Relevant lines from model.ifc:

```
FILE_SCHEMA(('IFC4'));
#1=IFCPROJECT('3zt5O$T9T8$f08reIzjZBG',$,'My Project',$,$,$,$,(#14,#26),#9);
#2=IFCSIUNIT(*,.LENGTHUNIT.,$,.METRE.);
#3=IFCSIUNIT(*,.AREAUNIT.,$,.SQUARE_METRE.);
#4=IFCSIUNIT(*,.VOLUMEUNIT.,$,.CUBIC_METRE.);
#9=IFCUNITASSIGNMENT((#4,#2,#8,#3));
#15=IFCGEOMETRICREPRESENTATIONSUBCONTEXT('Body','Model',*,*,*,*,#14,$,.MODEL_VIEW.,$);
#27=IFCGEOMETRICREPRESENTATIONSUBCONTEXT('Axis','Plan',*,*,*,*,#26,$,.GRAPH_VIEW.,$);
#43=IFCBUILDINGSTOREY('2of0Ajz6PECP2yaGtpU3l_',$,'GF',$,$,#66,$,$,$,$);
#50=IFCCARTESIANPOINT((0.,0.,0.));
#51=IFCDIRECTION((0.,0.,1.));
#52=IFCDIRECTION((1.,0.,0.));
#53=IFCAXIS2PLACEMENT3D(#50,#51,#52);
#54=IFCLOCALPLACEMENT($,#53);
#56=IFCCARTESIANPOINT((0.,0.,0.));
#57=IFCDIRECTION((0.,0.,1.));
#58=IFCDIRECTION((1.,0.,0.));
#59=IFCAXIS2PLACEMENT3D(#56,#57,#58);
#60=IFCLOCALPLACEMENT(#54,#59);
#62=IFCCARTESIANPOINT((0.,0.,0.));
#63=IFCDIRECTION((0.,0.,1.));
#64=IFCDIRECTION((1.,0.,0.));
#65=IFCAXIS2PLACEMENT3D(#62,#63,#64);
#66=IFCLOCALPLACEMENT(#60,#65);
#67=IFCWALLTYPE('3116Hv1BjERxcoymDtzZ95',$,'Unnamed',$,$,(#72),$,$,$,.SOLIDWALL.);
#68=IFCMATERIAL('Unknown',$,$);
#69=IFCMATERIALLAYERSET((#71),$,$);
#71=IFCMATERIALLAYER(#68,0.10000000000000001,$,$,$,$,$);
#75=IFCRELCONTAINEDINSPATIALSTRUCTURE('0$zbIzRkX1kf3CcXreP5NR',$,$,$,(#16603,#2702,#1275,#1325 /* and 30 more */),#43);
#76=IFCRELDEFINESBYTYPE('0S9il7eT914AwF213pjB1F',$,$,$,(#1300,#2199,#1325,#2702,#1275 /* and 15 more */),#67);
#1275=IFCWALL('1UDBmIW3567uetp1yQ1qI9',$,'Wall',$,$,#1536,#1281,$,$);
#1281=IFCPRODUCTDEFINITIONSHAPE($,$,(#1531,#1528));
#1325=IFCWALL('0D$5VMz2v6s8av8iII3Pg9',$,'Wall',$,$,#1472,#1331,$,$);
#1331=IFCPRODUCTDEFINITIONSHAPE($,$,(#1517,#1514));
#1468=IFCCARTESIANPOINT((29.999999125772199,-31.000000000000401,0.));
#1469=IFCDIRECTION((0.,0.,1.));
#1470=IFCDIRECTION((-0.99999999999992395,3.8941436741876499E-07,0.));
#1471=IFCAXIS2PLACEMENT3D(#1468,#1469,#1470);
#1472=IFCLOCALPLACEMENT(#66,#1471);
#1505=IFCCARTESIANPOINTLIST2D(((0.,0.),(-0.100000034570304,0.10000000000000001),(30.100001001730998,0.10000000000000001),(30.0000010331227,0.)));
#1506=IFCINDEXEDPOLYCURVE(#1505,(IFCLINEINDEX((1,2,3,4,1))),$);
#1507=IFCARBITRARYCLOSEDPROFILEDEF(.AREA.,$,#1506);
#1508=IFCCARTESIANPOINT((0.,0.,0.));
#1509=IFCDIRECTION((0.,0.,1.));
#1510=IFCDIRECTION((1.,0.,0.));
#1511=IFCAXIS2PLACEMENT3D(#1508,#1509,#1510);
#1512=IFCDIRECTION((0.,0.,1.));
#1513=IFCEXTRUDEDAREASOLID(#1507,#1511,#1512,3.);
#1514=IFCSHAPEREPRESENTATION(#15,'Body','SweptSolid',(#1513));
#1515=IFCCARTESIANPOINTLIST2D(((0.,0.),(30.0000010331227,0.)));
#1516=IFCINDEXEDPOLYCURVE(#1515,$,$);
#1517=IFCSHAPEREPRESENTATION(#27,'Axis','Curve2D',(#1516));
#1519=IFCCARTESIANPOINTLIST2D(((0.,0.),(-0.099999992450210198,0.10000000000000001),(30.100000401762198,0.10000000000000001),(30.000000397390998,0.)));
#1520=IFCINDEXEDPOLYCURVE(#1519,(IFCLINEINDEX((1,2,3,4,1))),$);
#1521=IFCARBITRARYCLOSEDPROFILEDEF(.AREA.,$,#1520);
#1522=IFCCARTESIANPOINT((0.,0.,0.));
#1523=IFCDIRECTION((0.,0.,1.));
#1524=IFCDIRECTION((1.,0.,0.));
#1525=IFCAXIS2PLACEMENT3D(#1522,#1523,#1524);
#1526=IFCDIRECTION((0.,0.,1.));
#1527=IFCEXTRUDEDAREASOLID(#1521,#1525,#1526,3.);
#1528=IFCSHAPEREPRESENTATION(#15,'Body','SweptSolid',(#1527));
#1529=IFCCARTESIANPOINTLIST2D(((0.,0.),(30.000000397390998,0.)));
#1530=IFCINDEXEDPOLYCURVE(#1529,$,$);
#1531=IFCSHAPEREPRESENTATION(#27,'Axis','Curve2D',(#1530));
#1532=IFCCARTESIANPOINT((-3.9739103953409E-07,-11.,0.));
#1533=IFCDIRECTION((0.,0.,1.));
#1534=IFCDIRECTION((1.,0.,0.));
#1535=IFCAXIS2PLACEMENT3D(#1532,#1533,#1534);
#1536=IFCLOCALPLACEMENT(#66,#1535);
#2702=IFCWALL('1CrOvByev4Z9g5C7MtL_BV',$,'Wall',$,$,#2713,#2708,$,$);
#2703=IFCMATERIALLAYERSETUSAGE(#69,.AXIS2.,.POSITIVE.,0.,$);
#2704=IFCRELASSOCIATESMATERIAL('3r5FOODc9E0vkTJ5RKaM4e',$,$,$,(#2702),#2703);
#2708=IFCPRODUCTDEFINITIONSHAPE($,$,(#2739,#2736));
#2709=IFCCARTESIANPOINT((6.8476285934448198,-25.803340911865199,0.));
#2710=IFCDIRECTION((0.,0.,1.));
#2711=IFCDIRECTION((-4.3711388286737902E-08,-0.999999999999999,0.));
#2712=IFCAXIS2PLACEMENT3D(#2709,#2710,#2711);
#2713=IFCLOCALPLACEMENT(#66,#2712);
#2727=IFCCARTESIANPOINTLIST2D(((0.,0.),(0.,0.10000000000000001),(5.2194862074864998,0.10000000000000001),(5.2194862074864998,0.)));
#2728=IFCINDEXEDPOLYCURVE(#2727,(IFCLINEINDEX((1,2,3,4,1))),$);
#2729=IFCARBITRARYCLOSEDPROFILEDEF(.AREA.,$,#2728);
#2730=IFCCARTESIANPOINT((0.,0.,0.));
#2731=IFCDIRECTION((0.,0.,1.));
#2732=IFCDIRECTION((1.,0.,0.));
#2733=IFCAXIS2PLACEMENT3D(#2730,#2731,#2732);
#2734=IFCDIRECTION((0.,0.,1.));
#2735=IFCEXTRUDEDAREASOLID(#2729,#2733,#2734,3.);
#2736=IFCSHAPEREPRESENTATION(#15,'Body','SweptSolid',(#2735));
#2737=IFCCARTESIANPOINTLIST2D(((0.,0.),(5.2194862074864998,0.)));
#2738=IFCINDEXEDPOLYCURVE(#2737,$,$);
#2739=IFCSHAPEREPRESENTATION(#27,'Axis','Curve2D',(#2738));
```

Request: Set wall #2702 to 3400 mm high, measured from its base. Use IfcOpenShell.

```python
import ifcopenshell
import ifcopenshell.geom
import ifcopenshell.util.representation
import ifcopenshell.util.shape
import ifcopenshell.util.unit

model = ifcopenshell.open("model.ifc")
unit_scale = ifcopenshell.util.unit.calculate_unit_scale(model)
settings = ifcopenshell.geom.settings()


def volume(element):
    """Net volume in cubic metres, openings subtracted."""
    shape = ifcopenshell.geom.create_shape(settings, element)
    return ifcopenshell.util.shape.get_volume(shape.geometry)


wall = model.by_guid("1CrOvByev4Z9g5C7MtL_BV")
before = volume(wall)

body = ifcopenshell.util.representation.get_representation(wall, "Model", "Body")
solid = body.Items[0]
old_height = solid.Depth
solid.Depth = 3.4 / unit_scale
after = volume(wall)

print(f"height {old_height:g} -> {solid.Depth:g}, volume {before:.3f} -> {after:.3f} m3")

model.write("model_rev.ifc")
```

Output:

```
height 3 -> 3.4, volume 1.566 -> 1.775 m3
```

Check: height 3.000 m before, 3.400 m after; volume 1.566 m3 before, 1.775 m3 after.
